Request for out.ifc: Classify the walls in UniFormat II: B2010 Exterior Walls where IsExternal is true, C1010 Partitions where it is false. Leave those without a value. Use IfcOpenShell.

First a look at what the model holds.

```python
import ifcopenshell
import ifcopenshell.util.element

model = ifcopenshell.open("out.ifc")
print(model.schema)
print("classifications:", [c.Name for c in model.by_type("IfcClassification")])
values = [ifcopenshell.util.element.get_pset(e, "Pset_WallCommon", "IsExternal") for e in model.by_type("IfcWall")]
for value in (True, False, None):
    print("IsExternal", value, values.count(value))
```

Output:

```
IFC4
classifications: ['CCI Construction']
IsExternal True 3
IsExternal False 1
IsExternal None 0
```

```python
import ifcopenshell
import ifcopenshell.api.classification
import ifcopenshell.util.element

model = ifcopenshell.open("out.ifc")

system = ifcopenshell.api.classification.add_classification(model, classification="UniFormat II")

walls = model.by_type("IfcWall")
external = {e: ifcopenshell.util.element.get_pset(e, "Pset_WallCommon", "IsExternal") for e in walls}
for flag, code, name in ((True, "B2010", "Exterior Walls"), (False, "C1010", "Partitions")):
    products = [e for e in walls if external[e] is flag]
    ifcopenshell.api.classification.add_reference(
        model, products=products, classification=system, identification=code, name=name
    )
    print(code, len(products))

model.write("out-out.ifc")
```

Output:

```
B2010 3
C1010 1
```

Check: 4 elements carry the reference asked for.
